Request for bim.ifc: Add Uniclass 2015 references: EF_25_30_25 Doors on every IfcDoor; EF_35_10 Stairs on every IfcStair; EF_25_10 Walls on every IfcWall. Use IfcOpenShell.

First a look at what the model holds.

```python
import ifcopenshell

model = ifcopenshell.open("bim.ifc")
print(model.schema)
print("classifications:", [c.Name for c in model.by_type("IfcClassification")])
for ifc_class in ("IfcDoor", "IfcRoof", "IfcStair", "IfcWall", "IfcWindow"):
    print(ifc_class, len(model.by_type(ifc_class)))
```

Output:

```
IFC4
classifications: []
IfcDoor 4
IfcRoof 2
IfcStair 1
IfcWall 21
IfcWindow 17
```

```python
import ifcopenshell
import ifcopenshell.api.classification

model = ifcopenshell.open("bim.ifc")

system = ifcopenshell.api.classification.add_classification(model, classification="Uniclass 2015")

codes = {
    "IfcDoor": ("EF_25_30_25", "Doors"),
    "IfcStair": ("EF_35_10", "Stairs"),
    "IfcWall": ("EF_25_10", "Walls"),
}
for ifc_class, (code, name) in codes.items():
    products = model.by_type(ifc_class)
    ifcopenshell.api.classification.add_reference(
        model, products=products, classification=system, identification=code, name=name
    )
    print(code, len(products))

model.write("bim_v2.ifc")
```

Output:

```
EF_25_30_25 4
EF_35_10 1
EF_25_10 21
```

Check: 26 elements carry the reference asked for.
